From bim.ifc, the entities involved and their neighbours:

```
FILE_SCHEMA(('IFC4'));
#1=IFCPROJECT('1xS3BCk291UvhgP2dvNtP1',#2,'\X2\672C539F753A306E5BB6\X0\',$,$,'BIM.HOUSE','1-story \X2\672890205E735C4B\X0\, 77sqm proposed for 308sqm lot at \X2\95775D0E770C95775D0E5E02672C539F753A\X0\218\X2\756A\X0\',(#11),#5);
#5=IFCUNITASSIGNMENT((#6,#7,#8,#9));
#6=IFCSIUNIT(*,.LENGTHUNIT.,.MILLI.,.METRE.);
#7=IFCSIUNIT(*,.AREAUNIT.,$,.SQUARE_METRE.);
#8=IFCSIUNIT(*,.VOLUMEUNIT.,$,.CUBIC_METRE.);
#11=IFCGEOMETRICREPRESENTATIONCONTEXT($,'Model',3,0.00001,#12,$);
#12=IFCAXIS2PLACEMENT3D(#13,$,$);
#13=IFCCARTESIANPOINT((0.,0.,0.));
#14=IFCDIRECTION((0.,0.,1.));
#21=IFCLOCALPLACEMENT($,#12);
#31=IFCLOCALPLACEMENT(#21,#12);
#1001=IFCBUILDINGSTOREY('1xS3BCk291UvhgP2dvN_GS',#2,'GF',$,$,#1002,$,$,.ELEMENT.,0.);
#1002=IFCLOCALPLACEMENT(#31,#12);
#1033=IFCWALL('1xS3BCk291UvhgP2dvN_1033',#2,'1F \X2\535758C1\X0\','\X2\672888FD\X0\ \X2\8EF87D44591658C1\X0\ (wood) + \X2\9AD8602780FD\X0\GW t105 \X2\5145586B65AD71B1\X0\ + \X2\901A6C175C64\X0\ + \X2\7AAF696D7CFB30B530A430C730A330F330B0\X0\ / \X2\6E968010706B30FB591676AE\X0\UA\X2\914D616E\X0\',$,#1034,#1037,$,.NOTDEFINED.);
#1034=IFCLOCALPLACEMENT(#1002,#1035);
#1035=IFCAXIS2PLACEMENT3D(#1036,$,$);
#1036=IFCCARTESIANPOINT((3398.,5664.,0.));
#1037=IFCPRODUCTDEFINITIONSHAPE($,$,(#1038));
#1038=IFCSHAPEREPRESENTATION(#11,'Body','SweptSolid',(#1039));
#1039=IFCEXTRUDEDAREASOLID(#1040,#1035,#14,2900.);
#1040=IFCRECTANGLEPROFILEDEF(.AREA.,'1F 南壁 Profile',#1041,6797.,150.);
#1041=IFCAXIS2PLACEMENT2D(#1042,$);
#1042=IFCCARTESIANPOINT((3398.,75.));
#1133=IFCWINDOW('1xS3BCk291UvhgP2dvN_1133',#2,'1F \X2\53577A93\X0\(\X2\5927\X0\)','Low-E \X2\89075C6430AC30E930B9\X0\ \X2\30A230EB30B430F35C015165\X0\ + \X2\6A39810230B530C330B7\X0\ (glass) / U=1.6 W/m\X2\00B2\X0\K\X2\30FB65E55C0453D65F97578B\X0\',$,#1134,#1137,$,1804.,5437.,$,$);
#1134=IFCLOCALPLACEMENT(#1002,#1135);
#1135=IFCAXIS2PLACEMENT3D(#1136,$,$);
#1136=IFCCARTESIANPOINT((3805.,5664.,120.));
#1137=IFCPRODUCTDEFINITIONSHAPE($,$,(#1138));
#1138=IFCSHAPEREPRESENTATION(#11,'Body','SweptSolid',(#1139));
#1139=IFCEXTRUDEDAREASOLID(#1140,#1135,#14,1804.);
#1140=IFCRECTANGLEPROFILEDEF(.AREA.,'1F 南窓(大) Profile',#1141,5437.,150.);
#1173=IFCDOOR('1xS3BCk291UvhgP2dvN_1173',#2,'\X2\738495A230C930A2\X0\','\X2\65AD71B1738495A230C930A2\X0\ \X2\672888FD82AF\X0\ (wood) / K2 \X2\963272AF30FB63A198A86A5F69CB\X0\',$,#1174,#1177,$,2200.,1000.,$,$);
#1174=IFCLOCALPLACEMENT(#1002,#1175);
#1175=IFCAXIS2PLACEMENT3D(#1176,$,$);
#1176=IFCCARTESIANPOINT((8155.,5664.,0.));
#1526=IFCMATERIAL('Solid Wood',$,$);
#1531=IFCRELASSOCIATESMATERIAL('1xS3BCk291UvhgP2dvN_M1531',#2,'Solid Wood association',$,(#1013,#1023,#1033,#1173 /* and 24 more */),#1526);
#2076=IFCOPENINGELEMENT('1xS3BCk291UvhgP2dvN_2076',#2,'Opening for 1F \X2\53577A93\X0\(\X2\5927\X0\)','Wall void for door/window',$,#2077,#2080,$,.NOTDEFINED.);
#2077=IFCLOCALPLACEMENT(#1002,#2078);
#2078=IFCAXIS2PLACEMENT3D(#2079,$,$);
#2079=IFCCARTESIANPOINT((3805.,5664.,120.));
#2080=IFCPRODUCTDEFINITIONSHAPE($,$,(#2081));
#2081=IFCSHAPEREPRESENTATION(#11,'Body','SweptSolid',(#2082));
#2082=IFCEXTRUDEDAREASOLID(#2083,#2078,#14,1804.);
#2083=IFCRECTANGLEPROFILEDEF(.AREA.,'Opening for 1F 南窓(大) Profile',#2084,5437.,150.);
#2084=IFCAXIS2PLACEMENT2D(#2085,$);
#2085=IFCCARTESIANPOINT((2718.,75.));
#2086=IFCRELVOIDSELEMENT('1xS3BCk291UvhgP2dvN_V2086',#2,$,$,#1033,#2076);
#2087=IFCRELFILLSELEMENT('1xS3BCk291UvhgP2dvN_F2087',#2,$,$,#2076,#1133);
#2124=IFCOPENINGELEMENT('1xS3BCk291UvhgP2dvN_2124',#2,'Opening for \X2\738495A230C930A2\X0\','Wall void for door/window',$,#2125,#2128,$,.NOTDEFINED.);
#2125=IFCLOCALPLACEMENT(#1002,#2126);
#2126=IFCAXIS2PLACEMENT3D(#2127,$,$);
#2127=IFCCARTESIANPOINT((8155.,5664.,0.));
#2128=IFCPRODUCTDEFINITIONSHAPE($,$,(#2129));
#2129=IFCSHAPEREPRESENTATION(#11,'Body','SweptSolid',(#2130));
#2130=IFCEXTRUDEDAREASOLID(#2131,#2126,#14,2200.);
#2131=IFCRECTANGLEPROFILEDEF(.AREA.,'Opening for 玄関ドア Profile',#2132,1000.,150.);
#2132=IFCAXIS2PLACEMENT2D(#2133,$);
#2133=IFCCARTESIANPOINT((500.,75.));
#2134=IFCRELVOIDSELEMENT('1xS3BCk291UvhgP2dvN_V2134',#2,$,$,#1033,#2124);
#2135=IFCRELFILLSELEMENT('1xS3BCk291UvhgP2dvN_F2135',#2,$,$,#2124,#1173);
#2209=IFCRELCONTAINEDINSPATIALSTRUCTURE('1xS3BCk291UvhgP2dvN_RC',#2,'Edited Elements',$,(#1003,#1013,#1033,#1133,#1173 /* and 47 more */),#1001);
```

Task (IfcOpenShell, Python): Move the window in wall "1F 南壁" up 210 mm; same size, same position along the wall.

```python
import numpy as np
import ifcopenshell
import ifcopenshell.api.geometry
import ifcopenshell.util.placement
import ifcopenshell.util.unit

model = ifcopenshell.open("bim.ifc")
unit_scale = ifcopenshell.util.unit.calculate_unit_scale(model)

window = model.by_guid("1xS3BCk291UvhgP2dvN_1133")
opening = window.FillsVoids[0].RelatingOpeningElement
dz = 0.21 / unit_scale

shift = np.array([0.0, 0.0, dz])
# The window is not placed relative to its opening, so move both.
for product in (opening, window):
    matrix = ifcopenshell.util.placement.get_local_placement(product.ObjectPlacement)
    matrix[:3, 3] += shift
    ifcopenshell.api.geometry.edit_object_placement(model, product=product, matrix=matrix, is_si=False)

print(f"moved by {dz * unit_scale:+.3f} m")

model.write("bim_updated.ifc")
```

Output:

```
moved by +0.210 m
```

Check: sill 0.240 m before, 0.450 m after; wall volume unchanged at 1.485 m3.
